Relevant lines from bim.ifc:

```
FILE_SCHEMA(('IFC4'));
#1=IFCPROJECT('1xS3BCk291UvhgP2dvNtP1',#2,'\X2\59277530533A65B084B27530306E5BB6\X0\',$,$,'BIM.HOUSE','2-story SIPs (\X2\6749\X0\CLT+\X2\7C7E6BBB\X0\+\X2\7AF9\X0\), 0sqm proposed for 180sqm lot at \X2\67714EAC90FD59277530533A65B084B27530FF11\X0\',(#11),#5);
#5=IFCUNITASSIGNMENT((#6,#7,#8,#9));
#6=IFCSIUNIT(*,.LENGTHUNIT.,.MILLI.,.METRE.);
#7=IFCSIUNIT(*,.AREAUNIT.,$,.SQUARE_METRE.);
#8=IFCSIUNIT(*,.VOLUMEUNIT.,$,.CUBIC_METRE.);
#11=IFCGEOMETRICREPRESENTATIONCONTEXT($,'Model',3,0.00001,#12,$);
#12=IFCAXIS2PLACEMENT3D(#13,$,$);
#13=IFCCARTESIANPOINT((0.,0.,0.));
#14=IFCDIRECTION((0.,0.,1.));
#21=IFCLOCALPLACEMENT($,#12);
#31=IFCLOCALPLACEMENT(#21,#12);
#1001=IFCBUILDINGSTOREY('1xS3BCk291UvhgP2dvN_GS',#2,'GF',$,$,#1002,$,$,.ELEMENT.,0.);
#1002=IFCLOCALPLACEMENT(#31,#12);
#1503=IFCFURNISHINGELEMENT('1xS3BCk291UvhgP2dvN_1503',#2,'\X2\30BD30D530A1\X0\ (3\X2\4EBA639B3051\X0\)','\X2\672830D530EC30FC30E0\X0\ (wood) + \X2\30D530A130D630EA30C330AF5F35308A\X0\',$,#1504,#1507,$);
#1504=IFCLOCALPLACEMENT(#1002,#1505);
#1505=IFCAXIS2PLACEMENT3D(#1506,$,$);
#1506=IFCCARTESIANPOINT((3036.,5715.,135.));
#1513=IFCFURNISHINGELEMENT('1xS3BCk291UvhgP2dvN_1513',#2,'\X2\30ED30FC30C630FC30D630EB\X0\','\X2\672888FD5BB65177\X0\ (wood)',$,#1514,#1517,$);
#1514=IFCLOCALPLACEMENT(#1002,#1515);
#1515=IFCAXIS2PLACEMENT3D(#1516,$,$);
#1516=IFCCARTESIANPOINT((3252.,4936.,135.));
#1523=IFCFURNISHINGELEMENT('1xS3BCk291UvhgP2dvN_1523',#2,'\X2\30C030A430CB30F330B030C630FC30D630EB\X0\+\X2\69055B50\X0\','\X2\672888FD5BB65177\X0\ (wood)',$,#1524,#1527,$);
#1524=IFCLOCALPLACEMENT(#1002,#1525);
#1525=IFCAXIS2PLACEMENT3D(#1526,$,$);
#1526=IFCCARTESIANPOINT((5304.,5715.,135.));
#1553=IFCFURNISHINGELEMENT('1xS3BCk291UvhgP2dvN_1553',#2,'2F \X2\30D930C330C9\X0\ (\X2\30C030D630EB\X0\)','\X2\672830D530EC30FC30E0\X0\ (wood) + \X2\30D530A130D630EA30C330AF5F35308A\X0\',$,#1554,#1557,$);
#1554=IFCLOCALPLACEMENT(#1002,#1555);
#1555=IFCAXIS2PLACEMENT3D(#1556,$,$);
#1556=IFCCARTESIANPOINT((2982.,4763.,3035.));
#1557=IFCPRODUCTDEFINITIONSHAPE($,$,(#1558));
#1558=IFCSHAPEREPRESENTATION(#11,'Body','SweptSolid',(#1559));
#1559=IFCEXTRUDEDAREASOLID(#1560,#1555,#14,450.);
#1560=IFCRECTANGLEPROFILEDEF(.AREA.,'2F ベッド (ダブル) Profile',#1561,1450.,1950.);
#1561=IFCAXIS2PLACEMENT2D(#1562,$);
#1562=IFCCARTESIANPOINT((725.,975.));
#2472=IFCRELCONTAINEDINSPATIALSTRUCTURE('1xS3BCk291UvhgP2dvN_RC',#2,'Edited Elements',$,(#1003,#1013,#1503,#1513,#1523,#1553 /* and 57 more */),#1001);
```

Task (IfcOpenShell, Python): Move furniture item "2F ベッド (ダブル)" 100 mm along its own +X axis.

```python
import ifcopenshell
import ifcopenshell.api.geometry
import ifcopenshell.util.placement

model = ifcopenshell.open("bim.ifc")

item = model.by_guid("1xS3BCk291UvhgP2dvN_1553")
matrix = ifcopenshell.util.placement.get_local_placement(item.ObjectPlacement)
matrix[:3, 3] += matrix[:3, 0] * 100.0
ifcopenshell.api.geometry.edit_object_placement(model, product=item, matrix=matrix, is_si=False)

print(ifcopenshell.util.placement.get_local_placement(item.ObjectPlacement).round(3) + 0.0)

model.write("bim-out.ifc")
```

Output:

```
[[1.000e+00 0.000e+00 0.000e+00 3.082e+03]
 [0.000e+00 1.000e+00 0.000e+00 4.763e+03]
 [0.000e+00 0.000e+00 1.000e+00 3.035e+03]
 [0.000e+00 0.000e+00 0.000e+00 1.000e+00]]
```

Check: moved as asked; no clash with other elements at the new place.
